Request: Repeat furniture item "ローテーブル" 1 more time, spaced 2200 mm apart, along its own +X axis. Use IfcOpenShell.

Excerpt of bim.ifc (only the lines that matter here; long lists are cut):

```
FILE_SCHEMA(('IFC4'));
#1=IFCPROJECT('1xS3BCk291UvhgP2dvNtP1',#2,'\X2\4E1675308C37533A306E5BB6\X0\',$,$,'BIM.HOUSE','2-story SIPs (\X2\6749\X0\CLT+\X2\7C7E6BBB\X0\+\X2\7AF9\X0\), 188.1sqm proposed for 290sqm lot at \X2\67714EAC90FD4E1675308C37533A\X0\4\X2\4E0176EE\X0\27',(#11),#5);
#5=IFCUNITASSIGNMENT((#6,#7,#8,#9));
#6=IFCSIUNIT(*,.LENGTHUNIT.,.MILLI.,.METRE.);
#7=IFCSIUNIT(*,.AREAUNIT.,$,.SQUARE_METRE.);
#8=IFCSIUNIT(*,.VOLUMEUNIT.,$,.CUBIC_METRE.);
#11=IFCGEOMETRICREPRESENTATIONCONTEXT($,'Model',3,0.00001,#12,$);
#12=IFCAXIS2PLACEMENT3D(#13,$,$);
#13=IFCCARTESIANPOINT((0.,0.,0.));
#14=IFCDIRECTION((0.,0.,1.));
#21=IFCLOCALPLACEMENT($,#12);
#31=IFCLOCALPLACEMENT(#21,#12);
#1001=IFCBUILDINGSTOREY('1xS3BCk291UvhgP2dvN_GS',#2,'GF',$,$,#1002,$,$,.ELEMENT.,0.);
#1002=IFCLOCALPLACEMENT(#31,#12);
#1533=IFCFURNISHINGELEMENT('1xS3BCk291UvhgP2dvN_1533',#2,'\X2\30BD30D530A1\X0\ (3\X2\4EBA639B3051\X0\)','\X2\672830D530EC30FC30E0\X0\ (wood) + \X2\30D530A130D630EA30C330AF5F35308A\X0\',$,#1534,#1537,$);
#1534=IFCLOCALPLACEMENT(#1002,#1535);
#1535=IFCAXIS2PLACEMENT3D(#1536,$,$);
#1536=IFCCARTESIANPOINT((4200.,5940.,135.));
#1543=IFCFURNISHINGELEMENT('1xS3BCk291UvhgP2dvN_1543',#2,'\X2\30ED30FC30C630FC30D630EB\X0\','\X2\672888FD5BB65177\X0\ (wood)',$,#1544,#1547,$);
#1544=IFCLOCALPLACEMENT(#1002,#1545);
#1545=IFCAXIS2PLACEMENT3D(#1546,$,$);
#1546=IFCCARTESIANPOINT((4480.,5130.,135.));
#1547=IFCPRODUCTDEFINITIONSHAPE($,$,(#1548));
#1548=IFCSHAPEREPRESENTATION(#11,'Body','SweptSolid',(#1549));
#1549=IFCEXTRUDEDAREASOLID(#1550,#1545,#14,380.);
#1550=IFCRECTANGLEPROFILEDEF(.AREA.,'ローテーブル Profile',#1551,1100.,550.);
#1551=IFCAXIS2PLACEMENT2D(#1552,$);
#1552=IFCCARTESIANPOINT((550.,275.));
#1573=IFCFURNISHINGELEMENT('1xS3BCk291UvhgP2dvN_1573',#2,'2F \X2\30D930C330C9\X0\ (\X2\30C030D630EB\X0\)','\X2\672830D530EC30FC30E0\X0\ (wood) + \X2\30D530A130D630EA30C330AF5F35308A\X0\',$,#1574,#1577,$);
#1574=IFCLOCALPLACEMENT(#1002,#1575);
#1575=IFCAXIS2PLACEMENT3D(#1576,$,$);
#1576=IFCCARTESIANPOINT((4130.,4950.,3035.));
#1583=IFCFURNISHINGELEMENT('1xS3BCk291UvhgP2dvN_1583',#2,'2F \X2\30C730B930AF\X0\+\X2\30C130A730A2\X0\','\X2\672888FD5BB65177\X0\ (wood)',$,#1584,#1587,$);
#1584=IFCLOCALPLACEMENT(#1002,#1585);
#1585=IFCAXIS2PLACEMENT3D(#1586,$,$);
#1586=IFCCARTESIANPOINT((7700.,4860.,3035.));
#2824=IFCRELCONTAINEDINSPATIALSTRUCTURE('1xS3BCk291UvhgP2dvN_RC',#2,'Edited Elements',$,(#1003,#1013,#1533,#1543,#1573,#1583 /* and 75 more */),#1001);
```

```python
import ifcopenshell
import ifcopenshell.api.geometry
import ifcopenshell.api.root
import ifcopenshell.util.element
import ifcopenshell.util.placement
import ifcopenshell.util.unit

model = ifcopenshell.open("bim.ifc")
unit_scale = ifcopenshell.util.unit.calculate_unit_scale(model)


def reuse_history(source, copy):
    """copy_class also copies each property set's owner history, people and application; keep the originals."""
    for rel in copy.IsDefinedBy:
        if rel.is_a("IfcRelDefinesByProperties") and (history := rel.RelatingPropertyDefinition.OwnerHistory):
            rel.RelatingPropertyDefinition.OwnerHistory = source.OwnerHistory
            ifcopenshell.util.element.remove_deep2(model, history)


source = model.by_guid("1xS3BCk291UvhgP2dvN_1543")
base = ifcopenshell.util.placement.get_local_placement(source.ObjectPlacement)
step = base[:3, 0] * 2.2 / unit_scale

for i in range(1, 2):
    copy = ifcopenshell.api.root.copy_class(model, product=source)
    copy.Representation = ifcopenshell.util.element.copy_deep(
        model, source.Representation, exclude=["IfcGeometricRepresentationContext", "IfcRepresentationMap"]
    )
    reuse_history(source, copy)
    matrix = base.copy()
    matrix[:3, 3] += i * step
    print("added at", matrix[:3, 3].round(3) + 0.0)
    ifcopenshell.api.geometry.edit_object_placement(model, product=copy, matrix=matrix, is_si=False)

model.write("bim_rev.ifc")
```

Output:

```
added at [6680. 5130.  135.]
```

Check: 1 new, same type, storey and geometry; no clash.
